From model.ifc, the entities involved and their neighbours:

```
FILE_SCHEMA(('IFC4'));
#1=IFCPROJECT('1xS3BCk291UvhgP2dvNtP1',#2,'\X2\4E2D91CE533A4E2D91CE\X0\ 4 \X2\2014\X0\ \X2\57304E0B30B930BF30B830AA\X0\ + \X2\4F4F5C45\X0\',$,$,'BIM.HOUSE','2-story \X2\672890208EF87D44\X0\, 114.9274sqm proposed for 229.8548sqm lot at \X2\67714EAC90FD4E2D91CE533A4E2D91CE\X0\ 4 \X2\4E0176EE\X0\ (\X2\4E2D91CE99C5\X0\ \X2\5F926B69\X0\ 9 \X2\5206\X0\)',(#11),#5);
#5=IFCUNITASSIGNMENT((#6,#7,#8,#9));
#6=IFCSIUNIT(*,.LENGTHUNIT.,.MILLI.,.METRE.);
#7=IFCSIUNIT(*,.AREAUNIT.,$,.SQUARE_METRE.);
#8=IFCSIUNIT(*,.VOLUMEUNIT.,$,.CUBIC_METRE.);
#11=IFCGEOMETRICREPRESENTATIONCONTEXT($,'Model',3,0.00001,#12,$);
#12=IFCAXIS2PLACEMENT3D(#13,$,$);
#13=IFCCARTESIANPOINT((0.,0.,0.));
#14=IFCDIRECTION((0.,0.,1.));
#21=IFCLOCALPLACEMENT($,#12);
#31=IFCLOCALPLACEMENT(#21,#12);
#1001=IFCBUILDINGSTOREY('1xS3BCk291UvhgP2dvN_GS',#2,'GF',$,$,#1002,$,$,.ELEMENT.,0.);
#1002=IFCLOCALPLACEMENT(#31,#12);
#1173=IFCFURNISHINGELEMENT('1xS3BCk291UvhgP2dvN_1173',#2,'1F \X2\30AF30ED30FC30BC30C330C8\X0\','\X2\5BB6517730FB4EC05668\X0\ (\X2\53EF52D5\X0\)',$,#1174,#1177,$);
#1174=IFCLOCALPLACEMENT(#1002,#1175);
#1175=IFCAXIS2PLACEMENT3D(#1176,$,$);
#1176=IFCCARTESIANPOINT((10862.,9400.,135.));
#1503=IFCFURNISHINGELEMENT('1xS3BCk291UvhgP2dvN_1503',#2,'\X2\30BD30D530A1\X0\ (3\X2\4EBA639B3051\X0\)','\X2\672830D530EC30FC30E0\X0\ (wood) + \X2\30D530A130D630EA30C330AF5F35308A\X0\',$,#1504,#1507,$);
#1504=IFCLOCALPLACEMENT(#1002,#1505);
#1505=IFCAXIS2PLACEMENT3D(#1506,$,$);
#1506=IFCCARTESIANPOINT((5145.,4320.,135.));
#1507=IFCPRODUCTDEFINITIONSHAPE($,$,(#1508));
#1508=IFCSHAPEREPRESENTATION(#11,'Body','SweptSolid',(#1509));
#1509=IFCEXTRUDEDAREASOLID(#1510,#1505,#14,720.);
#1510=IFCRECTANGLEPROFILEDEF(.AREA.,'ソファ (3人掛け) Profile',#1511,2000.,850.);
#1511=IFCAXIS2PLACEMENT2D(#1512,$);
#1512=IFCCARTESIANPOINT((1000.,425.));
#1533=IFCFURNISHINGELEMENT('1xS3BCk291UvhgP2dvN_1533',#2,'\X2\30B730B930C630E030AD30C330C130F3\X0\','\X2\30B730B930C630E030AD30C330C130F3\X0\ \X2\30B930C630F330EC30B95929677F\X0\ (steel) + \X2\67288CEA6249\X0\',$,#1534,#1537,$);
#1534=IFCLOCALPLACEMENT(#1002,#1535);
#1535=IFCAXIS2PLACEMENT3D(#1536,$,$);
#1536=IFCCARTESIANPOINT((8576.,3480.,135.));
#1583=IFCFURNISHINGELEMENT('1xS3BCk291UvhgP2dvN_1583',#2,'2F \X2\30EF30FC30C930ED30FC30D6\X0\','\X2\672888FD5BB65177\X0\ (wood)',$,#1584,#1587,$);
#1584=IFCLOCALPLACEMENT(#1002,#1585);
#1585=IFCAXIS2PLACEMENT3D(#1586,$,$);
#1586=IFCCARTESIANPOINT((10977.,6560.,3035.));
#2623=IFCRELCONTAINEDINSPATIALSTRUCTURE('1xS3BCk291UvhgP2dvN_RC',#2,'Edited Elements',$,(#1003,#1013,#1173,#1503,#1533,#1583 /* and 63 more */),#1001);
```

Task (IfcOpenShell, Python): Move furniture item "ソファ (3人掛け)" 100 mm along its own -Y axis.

```python
import ifcopenshell
import ifcopenshell.api.geometry
import ifcopenshell.util.placement

model = ifcopenshell.open("model.ifc")

item = model.by_id(1503)
matrix = ifcopenshell.util.placement.get_local_placement(item.ObjectPlacement)
matrix[:3, 3] -= matrix[:3, 1] * 100.0
ifcopenshell.api.geometry.edit_object_placement(model, product=item, matrix=matrix, is_si=False)

print(ifcopenshell.util.placement.get_local_placement(item.ObjectPlacement).round(3) + 0.0)

model.write("model_rev.ifc")
```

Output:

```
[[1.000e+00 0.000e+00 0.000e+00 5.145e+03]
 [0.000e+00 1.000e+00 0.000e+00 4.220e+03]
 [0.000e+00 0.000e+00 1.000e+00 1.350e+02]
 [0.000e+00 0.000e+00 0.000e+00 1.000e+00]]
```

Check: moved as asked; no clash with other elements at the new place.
